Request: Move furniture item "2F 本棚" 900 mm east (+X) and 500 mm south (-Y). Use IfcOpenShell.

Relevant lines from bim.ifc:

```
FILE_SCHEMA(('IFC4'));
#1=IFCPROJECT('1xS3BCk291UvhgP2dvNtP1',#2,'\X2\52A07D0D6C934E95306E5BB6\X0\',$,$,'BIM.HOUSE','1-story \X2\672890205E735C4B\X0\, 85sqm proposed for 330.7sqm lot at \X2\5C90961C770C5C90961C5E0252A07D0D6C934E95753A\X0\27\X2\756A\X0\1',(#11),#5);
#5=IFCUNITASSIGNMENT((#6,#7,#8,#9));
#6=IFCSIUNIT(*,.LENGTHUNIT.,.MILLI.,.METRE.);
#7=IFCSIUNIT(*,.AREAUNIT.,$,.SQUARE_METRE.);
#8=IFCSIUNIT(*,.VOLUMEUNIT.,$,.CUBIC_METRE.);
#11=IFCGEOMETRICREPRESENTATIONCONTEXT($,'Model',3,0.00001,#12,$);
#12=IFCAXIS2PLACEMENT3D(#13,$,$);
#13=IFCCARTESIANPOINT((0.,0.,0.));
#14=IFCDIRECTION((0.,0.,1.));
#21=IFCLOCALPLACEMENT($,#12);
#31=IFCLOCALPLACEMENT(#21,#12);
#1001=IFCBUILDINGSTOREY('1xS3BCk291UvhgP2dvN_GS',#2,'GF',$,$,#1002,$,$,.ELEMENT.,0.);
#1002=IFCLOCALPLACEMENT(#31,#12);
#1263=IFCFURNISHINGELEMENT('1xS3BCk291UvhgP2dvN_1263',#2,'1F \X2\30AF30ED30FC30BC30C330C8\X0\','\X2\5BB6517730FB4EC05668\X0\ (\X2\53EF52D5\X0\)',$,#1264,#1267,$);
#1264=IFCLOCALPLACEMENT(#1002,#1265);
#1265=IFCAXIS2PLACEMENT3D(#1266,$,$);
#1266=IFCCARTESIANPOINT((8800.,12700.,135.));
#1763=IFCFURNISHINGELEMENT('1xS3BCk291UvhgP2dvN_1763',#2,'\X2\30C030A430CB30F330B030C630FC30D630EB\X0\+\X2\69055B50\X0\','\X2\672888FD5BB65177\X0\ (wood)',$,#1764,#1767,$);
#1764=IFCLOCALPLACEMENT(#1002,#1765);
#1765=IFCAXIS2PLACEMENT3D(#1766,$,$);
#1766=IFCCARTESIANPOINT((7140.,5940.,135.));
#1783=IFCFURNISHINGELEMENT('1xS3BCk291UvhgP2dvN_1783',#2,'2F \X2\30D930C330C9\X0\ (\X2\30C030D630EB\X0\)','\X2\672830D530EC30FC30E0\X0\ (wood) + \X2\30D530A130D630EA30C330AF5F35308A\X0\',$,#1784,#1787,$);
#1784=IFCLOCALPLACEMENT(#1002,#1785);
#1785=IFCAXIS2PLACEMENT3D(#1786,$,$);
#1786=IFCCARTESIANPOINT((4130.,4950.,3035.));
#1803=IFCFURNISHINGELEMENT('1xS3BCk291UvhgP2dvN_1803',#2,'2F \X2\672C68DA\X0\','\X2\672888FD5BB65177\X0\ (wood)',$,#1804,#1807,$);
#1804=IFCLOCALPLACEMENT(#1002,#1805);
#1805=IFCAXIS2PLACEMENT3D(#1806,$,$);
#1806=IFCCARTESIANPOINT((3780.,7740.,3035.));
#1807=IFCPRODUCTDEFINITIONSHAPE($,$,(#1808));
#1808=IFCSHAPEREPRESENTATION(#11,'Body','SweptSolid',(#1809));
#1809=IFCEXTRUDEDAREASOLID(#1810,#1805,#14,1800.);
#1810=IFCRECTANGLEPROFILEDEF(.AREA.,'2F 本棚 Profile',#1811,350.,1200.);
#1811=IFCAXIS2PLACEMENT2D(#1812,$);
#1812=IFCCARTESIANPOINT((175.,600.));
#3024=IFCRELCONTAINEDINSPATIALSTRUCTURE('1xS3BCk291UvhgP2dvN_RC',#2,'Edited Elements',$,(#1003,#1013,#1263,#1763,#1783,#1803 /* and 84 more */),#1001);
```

```python
import ifcopenshell
import ifcopenshell.api.geometry
import ifcopenshell.util.placement
import ifcopenshell.util.unit

model = ifcopenshell.open("bim.ifc")
unit_scale = ifcopenshell.util.unit.calculate_unit_scale(model)

item = model.by_guid("1xS3BCk291UvhgP2dvN_1803")
matrix = ifcopenshell.util.placement.get_local_placement(item.ObjectPlacement)
matrix[0, 3] += 0.9 / unit_scale
matrix[1, 3] -= 0.5 / unit_scale
ifcopenshell.api.geometry.edit_object_placement(model, product=item, matrix=matrix, is_si=False)

print(ifcopenshell.util.placement.get_local_placement(item.ObjectPlacement).round(3) + 0.0)

model.write("bim-out.ifc")
```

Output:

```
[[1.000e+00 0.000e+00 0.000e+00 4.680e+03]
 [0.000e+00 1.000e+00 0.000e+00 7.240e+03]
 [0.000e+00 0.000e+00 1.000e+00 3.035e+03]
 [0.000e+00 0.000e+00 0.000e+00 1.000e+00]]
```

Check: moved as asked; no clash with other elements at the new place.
